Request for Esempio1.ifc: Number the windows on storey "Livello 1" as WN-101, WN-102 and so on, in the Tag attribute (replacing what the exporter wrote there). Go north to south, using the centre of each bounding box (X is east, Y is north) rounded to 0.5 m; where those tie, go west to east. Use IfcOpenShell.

First a look at what the model holds.

```python
import ifcopenshell
import ifcopenshell.util.element
import ifcopenshell.util.placement

model = ifcopenshell.open("Esempio1.ifc")
print(model.schema)
storey = next(s for s in model.by_type("IfcBuildingStorey") if s.Name == "Livello 1")
windows = [e for e in ifcopenshell.util.element.get_decomposition(storey) if e.is_a("IfcWindow")]
for e in sorted(windows, key=lambda e: e.id()):
    origin = ifcopenshell.util.placement.get_local_placement(e.ObjectPlacement)[:3, 3]
    print(e.id(), e.Tag, e.Name, origin.round(2) + 0.0, sep=" | ")
```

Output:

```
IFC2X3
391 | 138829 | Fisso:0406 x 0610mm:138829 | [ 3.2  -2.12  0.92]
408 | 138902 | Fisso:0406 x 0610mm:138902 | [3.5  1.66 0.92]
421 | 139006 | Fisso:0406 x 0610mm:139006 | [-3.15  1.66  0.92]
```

```python
import ifcopenshell
import ifcopenshell.geom
import ifcopenshell.util.element
import ifcopenshell.util.shape

model = ifcopenshell.open("Esempio1.ifc")
settings = ifcopenshell.geom.settings()
settings.set("use-world-coords", True)


def centre(element):
    shape = ifcopenshell.geom.create_shape(settings, element)
    return ifcopenshell.util.shape.get_bbox_centroid(shape.geometry)


storey = next(s for s in model.by_type("IfcBuildingStorey") if s.Name == "Livello 1")
windows = [e for e in ifcopenshell.util.element.get_decomposition(storey) if e.is_a("IfcWindow")]

# Insertion points can sit at a corner or the storey origin, so sort by the geometry (in metres).
centres = {e: centre(e) for e in windows}
windows.sort(key=lambda e: (-round(centres[e][1] / 0.5), centres[e][0]))

for i, e in enumerate(windows, start=1):
    number = f"WN-1{i:02d}"
    e.Tag = number
    print(e.id(), number)

model.write("Esempio1_v2.ifc")
```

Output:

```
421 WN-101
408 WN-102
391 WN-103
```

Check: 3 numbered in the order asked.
